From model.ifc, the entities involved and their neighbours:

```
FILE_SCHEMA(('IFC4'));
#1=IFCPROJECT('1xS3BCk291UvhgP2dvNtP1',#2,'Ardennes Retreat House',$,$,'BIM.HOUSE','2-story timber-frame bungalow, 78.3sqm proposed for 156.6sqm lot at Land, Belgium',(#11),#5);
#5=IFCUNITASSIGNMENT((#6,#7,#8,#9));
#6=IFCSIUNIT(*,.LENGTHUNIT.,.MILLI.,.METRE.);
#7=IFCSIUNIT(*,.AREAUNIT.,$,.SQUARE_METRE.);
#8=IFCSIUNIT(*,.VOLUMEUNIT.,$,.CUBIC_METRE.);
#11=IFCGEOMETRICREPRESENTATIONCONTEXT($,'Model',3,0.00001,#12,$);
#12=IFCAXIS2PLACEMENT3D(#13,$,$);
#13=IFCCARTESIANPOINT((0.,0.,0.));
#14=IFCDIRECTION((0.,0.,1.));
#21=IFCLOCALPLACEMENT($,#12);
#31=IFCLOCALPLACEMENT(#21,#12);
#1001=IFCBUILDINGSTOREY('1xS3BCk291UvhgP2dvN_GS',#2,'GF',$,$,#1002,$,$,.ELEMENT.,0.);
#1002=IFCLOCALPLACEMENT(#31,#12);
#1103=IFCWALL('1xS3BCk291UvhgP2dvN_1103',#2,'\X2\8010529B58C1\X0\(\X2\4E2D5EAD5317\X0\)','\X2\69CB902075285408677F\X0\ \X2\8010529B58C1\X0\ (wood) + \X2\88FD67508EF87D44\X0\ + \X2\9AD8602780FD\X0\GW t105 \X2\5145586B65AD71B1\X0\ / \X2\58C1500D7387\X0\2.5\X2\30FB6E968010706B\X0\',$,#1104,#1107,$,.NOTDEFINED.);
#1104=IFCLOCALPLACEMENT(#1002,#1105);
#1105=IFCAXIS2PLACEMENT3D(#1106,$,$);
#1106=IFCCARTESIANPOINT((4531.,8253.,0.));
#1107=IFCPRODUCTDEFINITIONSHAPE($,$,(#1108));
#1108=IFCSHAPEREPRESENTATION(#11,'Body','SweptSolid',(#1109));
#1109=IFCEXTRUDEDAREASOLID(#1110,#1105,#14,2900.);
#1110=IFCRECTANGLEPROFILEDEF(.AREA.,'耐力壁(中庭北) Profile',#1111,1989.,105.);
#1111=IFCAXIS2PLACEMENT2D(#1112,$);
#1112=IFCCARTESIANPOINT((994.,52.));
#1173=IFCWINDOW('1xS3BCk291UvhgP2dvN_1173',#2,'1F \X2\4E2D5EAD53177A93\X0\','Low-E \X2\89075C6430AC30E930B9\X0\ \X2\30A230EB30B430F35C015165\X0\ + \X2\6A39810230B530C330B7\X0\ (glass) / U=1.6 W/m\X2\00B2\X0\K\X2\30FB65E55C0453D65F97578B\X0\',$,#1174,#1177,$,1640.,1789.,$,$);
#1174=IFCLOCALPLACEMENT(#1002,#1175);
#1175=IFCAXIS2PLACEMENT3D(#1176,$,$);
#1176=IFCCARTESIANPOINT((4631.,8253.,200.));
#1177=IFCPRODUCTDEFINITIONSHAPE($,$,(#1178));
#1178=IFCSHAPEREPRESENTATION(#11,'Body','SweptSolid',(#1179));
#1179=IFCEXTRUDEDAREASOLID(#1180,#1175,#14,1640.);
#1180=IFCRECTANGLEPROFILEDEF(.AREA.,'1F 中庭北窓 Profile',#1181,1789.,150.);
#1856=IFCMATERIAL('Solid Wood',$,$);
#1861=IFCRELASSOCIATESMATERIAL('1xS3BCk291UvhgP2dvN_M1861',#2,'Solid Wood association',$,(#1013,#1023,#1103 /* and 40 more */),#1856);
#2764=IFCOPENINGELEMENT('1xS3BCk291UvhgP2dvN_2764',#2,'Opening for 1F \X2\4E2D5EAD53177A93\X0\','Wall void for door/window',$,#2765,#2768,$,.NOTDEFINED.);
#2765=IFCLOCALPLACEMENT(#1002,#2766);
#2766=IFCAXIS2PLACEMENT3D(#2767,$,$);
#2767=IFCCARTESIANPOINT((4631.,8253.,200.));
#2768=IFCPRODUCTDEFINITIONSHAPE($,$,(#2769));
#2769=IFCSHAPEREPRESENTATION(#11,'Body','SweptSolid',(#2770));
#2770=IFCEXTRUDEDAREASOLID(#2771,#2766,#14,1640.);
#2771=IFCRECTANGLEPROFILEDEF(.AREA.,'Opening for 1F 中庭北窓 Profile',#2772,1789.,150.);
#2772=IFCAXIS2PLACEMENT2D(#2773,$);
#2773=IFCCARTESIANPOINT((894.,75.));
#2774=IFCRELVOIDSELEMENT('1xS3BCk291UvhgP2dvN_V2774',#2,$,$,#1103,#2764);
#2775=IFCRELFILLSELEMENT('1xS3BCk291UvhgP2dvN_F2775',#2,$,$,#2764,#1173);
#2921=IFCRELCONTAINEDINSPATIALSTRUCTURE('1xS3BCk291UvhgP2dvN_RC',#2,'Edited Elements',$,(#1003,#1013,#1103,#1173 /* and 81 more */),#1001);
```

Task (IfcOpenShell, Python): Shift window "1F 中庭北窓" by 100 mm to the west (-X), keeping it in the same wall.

```python
import ifcopenshell
import ifcopenshell.api.geometry
import ifcopenshell.util.placement

model = ifcopenshell.open("model.ifc")

window = model.by_guid("1xS3BCk291UvhgP2dvN_1173")
opening = window.FillsVoids[0].RelatingOpeningElement
wall = opening.VoidsElements[0].RelatingBuildingElement

wall_matrix = ifcopenshell.util.placement.get_local_placement(wall.ObjectPlacement)
shift = wall_matrix[:3, 0] * -100.0
before = ifcopenshell.util.placement.get_local_placement(window.ObjectPlacement)[:3, 3].copy()

# The window is not placed relative to its opening, so move both.
for product in (opening, window):
    matrix = ifcopenshell.util.placement.get_local_placement(product.ObjectPlacement)
    matrix[:3, 3] += shift
    ifcopenshell.api.geometry.edit_object_placement(model, product=product, matrix=matrix, is_si=False)

after = ifcopenshell.util.placement.get_local_placement(window.ObjectPlacement)[:3, 3]
print("window moved by", (after - before).round(3) + 0.0)

model.write("model_v2.ifc")
```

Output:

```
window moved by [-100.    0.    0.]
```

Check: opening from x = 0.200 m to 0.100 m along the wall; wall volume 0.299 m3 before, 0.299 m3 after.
